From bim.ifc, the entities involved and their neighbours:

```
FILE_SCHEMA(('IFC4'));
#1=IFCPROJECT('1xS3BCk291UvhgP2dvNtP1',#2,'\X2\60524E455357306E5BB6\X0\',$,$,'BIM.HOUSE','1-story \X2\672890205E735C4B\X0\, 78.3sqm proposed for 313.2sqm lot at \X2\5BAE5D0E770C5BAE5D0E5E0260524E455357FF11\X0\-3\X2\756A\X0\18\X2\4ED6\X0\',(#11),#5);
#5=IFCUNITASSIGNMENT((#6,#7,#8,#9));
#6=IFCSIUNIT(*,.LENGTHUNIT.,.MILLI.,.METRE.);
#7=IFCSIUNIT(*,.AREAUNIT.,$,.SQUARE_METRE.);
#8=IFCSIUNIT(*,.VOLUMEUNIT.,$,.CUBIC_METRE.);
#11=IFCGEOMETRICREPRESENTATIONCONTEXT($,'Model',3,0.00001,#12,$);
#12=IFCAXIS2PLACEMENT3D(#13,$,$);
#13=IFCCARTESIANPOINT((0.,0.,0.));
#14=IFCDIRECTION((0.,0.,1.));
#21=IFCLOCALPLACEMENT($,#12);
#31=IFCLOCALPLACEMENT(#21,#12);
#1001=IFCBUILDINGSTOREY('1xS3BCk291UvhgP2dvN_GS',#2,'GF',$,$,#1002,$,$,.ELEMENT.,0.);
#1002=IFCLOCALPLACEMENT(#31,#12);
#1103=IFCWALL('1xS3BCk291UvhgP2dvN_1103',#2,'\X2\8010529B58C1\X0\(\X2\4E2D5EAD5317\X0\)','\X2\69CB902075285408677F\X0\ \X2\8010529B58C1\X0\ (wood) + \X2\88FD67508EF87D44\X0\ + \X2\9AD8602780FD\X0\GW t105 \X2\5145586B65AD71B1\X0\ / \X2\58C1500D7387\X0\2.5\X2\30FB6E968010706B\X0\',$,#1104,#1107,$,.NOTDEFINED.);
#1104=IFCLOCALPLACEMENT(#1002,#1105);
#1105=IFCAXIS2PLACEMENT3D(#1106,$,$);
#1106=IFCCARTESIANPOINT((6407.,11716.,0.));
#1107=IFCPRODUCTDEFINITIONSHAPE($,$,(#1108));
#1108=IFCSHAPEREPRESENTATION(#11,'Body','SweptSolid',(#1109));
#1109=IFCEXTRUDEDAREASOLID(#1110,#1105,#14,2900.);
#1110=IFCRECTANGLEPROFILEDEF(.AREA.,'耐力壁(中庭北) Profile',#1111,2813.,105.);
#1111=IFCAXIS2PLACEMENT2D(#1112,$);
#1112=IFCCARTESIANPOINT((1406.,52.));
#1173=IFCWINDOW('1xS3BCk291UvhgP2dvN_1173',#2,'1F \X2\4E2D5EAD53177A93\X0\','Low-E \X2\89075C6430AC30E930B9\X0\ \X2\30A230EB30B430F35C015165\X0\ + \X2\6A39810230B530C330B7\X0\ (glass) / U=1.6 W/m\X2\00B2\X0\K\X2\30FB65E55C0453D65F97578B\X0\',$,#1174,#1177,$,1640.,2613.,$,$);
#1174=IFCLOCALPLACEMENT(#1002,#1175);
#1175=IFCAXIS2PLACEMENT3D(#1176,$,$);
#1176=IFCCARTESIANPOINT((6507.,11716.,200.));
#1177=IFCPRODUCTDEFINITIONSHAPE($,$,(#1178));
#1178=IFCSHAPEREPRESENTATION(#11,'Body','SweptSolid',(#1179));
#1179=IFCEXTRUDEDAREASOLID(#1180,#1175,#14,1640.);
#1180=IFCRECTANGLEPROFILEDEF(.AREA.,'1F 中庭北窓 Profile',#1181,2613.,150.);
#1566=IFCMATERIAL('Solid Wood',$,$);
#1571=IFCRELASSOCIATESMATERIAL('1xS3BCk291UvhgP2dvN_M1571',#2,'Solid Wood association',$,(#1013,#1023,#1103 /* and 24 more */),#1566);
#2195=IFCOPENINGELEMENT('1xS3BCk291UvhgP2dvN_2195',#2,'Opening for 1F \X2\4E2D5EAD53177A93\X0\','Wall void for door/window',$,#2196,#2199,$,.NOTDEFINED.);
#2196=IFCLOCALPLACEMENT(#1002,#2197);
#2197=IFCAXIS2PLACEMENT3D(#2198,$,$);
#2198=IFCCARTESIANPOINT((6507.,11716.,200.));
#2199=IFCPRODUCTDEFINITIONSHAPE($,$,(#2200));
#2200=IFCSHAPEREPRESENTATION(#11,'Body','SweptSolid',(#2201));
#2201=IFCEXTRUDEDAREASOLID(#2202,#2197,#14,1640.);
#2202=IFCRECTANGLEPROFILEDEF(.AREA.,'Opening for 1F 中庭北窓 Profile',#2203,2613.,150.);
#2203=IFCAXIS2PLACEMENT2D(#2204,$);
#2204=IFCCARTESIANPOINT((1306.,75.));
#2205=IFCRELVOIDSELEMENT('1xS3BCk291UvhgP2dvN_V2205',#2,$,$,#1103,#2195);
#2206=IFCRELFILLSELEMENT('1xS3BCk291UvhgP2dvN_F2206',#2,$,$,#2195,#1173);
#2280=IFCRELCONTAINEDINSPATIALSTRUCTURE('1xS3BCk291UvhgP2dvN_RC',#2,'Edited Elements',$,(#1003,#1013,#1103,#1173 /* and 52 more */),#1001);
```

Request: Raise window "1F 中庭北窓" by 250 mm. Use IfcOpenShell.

```python
import numpy as np
import ifcopenshell
import ifcopenshell.api.geometry
import ifcopenshell.util.placement
import ifcopenshell.util.unit

model = ifcopenshell.open("bim.ifc")
unit_scale = ifcopenshell.util.unit.calculate_unit_scale(model)

window = model.by_guid("1xS3BCk291UvhgP2dvN_1173")
opening = window.FillsVoids[0].RelatingOpeningElement
dz = 0.25 / unit_scale

shift = np.array([0.0, 0.0, dz])
# The window is not placed relative to its opening, so move both.
for product in (opening, window):
    matrix = ifcopenshell.util.placement.get_local_placement(product.ObjectPlacement)
    matrix[:3, 3] += shift
    ifcopenshell.api.geometry.edit_object_placement(model, product=product, matrix=matrix, is_si=False)

print(f"moved by {dz * unit_scale:+.3f} m")

model.write("bim_v2.ifc")
```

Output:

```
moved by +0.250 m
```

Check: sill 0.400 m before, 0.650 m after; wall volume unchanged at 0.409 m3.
